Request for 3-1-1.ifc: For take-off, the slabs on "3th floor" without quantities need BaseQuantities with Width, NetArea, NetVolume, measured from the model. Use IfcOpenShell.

First a look at what the model holds.

```python
import ifcopenshell
import ifcopenshell.util.element
import ifcopenshell.util.unit

model = ifcopenshell.open("3-1-1.ifc")
print(model.schema)
for unit_type in ("LENGTHUNIT", "AREAUNIT", "VOLUMEUNIT"):
    print(unit_type, ifcopenshell.util.unit.calculate_unit_scale(model, unit_type))
storey = next(s for s in model.by_type("IfcBuildingStorey") if s.Name == "3th floor")
slabs = [e for e in ifcopenshell.util.element.get_decomposition(storey) if e.is_a("IfcSlab")]
for e in sorted(slabs, key=lambda e: e.id()):
    print(e.id(), e.is_a(), e.Name, list(ifcopenshell.util.element.get_psets(e, qtos_only=True)), sep=" | ")
```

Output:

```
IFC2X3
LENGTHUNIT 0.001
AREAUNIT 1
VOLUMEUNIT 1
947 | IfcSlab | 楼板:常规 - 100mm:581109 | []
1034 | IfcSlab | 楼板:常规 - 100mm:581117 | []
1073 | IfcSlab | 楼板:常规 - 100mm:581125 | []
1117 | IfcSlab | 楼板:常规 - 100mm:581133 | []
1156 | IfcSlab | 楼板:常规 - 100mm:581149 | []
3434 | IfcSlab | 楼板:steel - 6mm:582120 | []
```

```python
import ifcopenshell
import ifcopenshell.api.pset
import ifcopenshell.geom
import ifcopenshell.util.element
import ifcopenshell.util.shape
import ifcopenshell.util.unit

model = ifcopenshell.open("3-1-1.ifc")
unit_scale = ifcopenshell.util.unit.calculate_unit_scale(model)
area_scale = ifcopenshell.util.unit.calculate_unit_scale(model, "AREAUNIT")
volume_scale = ifcopenshell.util.unit.calculate_unit_scale(model, "VOLUMEUNIT")
settings = ifcopenshell.geom.settings()

storey = next(s for s in model.by_type("IfcBuildingStorey") if s.Name == "3th floor")
slabs = [e for e in ifcopenshell.util.element.get_decomposition(storey) if e.is_a("IfcSlab")]

for e in sorted(slabs, key=lambda e: e.id()):
    if ifcopenshell.util.element.get_psets(e, qtos_only=True, should_inherit=False):
        continue
    # Geometry comes back in metres, in the element's own axes.
    shape = ifcopenshell.geom.create_shape(settings, e)
    values = {
        "Width": ifcopenshell.util.shape.get_z(shape.geometry) / unit_scale,
        "NetArea": ifcopenshell.util.shape.get_footprint_area(shape.geometry) / area_scale,
        "NetVolume": ifcopenshell.util.shape.get_volume(shape.geometry) / volume_scale,
    }
    qto = ifcopenshell.api.pset.add_qto(model, product=e, name="BaseQuantities")
    ifcopenshell.api.pset.edit_qto(model, qto=qto, properties=values)
    print(e.id(), {k: round(v, 3) for k, v in values.items()})

model.write("3-1-1_v2.ifc")
```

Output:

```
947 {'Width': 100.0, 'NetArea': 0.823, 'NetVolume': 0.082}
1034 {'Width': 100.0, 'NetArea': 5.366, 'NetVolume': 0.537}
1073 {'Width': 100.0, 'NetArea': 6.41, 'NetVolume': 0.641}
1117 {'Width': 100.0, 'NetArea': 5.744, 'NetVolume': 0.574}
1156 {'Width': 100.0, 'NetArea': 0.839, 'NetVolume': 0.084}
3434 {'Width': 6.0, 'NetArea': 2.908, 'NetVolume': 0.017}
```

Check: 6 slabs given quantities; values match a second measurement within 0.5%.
